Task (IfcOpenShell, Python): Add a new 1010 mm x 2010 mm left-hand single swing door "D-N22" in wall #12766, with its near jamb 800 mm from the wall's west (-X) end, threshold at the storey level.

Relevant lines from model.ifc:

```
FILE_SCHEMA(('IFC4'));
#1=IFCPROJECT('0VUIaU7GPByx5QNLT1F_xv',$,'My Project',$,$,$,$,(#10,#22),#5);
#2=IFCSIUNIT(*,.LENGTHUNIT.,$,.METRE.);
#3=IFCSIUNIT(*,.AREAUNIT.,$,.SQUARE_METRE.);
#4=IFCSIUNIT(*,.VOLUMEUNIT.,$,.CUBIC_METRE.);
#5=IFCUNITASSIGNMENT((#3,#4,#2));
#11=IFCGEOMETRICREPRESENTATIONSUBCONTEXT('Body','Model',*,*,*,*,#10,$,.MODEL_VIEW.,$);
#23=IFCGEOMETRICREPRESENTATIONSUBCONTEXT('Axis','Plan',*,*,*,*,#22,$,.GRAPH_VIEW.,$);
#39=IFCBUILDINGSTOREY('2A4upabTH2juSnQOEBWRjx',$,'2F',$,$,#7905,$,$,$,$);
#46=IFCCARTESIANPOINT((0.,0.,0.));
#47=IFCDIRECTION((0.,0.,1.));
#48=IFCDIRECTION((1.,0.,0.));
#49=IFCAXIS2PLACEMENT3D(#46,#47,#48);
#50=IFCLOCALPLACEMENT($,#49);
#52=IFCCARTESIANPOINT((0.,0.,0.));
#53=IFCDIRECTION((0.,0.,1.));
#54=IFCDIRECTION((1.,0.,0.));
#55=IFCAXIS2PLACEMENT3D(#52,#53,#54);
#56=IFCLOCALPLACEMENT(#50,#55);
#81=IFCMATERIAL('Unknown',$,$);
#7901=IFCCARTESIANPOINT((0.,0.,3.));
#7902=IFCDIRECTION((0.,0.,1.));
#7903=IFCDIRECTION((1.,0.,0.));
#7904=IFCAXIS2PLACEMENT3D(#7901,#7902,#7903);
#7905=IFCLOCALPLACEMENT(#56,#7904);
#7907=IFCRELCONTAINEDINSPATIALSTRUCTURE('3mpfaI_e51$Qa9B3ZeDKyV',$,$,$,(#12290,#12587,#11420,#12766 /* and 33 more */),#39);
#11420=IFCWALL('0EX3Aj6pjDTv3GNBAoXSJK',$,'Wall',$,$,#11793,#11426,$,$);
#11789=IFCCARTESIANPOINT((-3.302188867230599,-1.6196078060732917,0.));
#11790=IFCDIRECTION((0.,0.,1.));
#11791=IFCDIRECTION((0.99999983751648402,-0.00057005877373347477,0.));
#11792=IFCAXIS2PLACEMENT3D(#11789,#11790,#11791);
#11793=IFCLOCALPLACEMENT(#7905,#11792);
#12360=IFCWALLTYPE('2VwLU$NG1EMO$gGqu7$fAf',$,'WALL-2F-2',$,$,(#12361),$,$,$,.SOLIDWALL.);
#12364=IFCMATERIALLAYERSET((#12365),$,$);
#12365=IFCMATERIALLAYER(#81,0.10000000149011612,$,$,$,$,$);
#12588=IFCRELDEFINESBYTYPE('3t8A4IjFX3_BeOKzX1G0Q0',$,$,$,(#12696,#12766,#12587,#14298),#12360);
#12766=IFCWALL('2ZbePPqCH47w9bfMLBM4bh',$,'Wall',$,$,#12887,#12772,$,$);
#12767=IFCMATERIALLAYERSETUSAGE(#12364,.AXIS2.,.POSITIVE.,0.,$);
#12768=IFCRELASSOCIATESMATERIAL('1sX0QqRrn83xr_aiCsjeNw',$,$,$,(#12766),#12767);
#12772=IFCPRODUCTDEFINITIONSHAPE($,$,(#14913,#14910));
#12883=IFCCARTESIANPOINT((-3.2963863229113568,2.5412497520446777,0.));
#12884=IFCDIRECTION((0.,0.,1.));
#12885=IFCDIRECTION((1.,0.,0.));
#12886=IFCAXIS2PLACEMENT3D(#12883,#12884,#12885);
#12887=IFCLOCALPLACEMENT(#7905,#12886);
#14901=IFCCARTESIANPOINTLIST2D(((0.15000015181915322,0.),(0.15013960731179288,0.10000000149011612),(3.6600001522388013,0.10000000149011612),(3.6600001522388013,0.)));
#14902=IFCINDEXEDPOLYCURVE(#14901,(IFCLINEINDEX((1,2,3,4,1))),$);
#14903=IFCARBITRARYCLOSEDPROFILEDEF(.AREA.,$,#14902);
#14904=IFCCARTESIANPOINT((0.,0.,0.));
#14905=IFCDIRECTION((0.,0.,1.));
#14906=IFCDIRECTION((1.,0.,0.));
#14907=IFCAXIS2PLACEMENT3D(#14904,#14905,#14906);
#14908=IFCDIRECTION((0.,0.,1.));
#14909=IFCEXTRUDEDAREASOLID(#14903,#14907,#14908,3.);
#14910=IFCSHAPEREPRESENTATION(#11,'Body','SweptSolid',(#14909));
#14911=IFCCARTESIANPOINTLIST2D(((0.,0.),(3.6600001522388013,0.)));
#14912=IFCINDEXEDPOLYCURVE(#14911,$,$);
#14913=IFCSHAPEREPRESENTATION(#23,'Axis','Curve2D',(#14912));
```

```python
import numpy as np
import ifcopenshell
import ifcopenshell.api.feature
import ifcopenshell.api.geometry
import ifcopenshell.api.root
import ifcopenshell.api.spatial
import ifcopenshell.geom
import ifcopenshell.util.element
import ifcopenshell.util.placement
import ifcopenshell.util.representation
import ifcopenshell.util.shape
import ifcopenshell.util.unit

model = ifcopenshell.open("model.ifc")
unit_scale = ifcopenshell.util.unit.calculate_unit_scale(model)
settings = ifcopenshell.geom.settings()


def volume(element):
    """Net volume in cubic metres, openings subtracted."""
    shape = ifcopenshell.geom.create_shape(settings, element)
    return ifcopenshell.util.shape.get_volume(shape.geometry)


wall = model.by_guid("2ZbePPqCH47w9bfMLBM4bh")
storey = ifcopenshell.util.element.get_container(wall, ifc_class="IfcBuildingStorey")
context = ifcopenshell.util.representation.get_context(model, "Model", "Body", "MODEL_VIEW")
before = volume(wall)

width, height, from_end, sill = 1.01, 2.01, 0.8, 0.0  # metres

# The wall runs along its own X axis, and the end named is its -X end.
wall_shape = ifcopenshell.geom.create_shape(settings, wall)
x, y, z = ifcopenshell.util.shape.get_vertices(wall_shape.geometry).T
start = x.min() + from_end
face, thickness = float(y.min()), float(y.max() - y.min())
wall_matrix = ifcopenshell.util.placement.get_local_placement(wall.ObjectPlacement)
level = ifcopenshell.util.placement.get_local_placement(storey.ObjectPlacement)[2, 3]


def in_wall(x, y):
    """Placement at x, y metres in the wall's axes, at sill height."""
    matrix = wall_matrix.copy()
    matrix[:, 3] = wall_matrix @ np.array([x / unit_scale, y / unit_scale, 0.0, 1.0])
    matrix[2, 3] = level + sill / unit_scale
    return matrix


# Opening: a box that overshoots both wall faces by 50 mm.
opening = ifcopenshell.api.root.create_entity(model, ifc_class="IfcOpeningElement", predefined_type="OPENING")
box = ifcopenshell.api.geometry.add_wall_representation(
    model, context=context, length=width, height=height, thickness=thickness + 0.1
)
ifcopenshell.api.geometry.assign_representation(model, product=opening, representation=box)
ifcopenshell.api.geometry.edit_object_placement(model, product=opening, matrix=in_wall(start, face - 0.05), is_si=False)
ifcopenshell.api.feature.add_feature(model, feature=opening, element=wall)

door = ifcopenshell.api.root.create_entity(model, ifc_class="IfcDoor", name="D-N22", predefined_type="DOOR")
door.OverallWidth, door.OverallHeight = width / unit_scale, height / unit_scale
door.OperationType = "SINGLE_SWING_LEFT"
body = ifcopenshell.api.geometry.add_door_representation(
    model,
    context=context,
    overall_width=door.OverallWidth,
    overall_height=door.OverallHeight,
    operation_type="SINGLE_SWING_LEFT",
    lining_properties={"LiningDepth": thickness / unit_scale, "ThresholdDepth": thickness / unit_scale},
)
ifcopenshell.api.geometry.assign_representation(model, product=door, representation=body)
ifcopenshell.api.spatial.assign_container(model, products=[door], relating_structure=storey)
ifcopenshell.api.feature.add_filling(model, opening=opening, element=door)

# The lining spans the wall, so the door starts at the wall face.
ifcopenshell.api.geometry.edit_object_placement(model, product=door, matrix=in_wall(start, face), is_si=False)

after = volume(wall)

print(f"wall volume {before:.3f} -> {after:.3f} m3")

model.write("model_edited.ifc")
```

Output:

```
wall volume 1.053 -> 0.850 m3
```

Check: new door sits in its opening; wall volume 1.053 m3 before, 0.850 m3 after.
